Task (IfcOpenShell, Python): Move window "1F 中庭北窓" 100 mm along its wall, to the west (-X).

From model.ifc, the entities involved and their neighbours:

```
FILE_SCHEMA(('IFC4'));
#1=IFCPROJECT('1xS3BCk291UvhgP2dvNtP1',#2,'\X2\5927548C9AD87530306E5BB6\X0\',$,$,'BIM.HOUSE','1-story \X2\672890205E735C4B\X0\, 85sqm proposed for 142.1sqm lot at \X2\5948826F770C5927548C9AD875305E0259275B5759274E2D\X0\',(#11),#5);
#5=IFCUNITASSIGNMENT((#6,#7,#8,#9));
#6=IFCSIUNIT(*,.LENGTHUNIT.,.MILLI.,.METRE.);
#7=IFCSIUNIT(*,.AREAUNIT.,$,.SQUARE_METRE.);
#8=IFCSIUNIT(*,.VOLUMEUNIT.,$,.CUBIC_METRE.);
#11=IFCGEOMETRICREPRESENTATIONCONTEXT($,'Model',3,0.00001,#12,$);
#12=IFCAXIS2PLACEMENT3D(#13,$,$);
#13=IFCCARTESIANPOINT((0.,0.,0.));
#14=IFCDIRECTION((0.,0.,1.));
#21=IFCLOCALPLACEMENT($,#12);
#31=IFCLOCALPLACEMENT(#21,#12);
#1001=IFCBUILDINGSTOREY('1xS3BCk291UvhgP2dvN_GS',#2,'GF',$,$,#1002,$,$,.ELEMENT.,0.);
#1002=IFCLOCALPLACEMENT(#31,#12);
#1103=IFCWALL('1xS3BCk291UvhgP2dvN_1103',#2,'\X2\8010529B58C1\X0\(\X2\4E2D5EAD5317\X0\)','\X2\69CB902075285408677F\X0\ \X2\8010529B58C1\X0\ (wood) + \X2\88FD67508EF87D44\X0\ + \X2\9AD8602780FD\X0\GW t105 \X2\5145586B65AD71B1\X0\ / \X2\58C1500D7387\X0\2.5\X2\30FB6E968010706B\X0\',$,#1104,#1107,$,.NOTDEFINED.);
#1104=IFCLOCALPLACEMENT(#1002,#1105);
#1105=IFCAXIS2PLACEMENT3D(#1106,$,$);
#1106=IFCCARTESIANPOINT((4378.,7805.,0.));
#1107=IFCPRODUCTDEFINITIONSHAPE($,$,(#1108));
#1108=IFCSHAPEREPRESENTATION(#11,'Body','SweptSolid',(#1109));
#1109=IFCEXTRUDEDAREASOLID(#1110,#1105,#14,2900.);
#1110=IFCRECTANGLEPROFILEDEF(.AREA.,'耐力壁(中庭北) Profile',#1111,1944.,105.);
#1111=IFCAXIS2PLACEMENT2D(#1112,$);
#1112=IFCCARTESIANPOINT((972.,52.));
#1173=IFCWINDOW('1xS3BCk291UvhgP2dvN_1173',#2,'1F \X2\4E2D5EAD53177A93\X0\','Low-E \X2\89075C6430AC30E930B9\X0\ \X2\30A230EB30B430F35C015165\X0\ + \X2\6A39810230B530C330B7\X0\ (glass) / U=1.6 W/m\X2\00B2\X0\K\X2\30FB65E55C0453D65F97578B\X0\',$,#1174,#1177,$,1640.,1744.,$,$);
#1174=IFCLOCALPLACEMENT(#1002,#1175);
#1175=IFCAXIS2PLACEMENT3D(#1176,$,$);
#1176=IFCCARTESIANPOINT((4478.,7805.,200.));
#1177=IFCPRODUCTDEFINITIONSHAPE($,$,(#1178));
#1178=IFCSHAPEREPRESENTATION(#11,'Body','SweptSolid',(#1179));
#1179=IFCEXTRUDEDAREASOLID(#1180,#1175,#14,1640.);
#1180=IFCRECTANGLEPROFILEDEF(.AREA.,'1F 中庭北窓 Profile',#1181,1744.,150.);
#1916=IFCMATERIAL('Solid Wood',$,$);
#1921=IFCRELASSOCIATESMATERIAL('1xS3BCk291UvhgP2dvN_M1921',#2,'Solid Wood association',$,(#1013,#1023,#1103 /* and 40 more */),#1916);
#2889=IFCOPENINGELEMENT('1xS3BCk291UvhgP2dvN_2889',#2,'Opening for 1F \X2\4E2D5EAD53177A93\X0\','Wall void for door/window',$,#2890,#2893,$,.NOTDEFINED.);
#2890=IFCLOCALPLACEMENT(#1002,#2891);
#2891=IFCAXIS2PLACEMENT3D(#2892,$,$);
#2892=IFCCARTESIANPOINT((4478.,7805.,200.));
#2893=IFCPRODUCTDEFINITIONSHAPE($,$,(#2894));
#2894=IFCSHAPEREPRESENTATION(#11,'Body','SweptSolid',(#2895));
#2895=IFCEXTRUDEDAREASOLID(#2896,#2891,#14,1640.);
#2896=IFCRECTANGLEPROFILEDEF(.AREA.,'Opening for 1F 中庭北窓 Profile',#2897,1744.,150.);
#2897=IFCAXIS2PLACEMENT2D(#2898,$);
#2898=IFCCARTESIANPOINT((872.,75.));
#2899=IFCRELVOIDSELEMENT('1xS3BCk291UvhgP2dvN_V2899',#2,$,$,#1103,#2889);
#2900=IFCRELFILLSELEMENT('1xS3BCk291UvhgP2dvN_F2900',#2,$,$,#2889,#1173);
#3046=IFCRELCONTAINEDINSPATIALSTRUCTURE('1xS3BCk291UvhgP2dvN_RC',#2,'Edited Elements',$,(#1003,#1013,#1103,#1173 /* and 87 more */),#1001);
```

```python
import ifcopenshell
import ifcopenshell.api.geometry
import ifcopenshell.util.placement

model = ifcopenshell.open("model.ifc")

window = model.by_id(1173)
opening = window.FillsVoids[0].RelatingOpeningElement
wall = opening.VoidsElements[0].RelatingBuildingElement

wall_matrix = ifcopenshell.util.placement.get_local_placement(wall.ObjectPlacement)
shift = wall_matrix[:3, 0] * -100.0
before = ifcopenshell.util.placement.get_local_placement(window.ObjectPlacement)[:3, 3].copy()

# The window is not placed relative to its opening, so move both.
for product in (opening, window):
    matrix = ifcopenshell.util.placement.get_local_placement(product.ObjectPlacement)
    matrix[:3, 3] += shift
    ifcopenshell.api.geometry.edit_object_placement(model, product=product, matrix=matrix, is_si=False)

after = ifcopenshell.util.placement.get_local_placement(window.ObjectPlacement)[:3, 3]
print("window moved by", (after - before).round(3) + 0.0)

model.write("model_updated.ifc")
```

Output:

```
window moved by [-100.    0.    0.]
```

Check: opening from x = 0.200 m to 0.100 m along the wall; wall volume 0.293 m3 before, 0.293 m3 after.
